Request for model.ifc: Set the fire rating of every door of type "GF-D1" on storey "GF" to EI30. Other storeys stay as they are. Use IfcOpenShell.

First a look at what the model holds.

```python
import ifcopenshell
import ifcopenshell.util.element

model = ifcopenshell.open("model.ifc")
print(model.schema)
storey = next(s for s in model.by_type("IfcBuildingStorey") if s.Name == "GF")
doors = [e for e in ifcopenshell.util.element.get_decomposition(storey) if e.is_a("IfcDoor")]
seen = {}
for e in doors:
    element_type = ifcopenshell.util.element.get_type(e)
    key = (element_type.Name if element_type != e and element_type else None, ifcopenshell.util.element.get_pset(e, "Pset_DoorCommon", "FireRating"))
    seen[key] = seen.get(key, 0) + 1
for (name, value), count in sorted(seen.items(), key=str):
    print(count, "x", name, "|", value)
```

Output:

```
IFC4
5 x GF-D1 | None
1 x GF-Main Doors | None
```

```python
import ifcopenshell
import ifcopenshell.api.pset
import ifcopenshell.util.element

model = ifcopenshell.open("model.ifc")

storey = next(s for s in model.by_type("IfcBuildingStorey") if s.Name == "GF")
doors = [e for e in ifcopenshell.util.element.get_decomposition(storey) if e.is_a("IfcDoor")]

count = 0
for e in doors:
    element_type = ifcopenshell.util.element.get_type(e)
    if element_type in (None, e) or element_type.Name != "GF-D1":
        continue
    # add_pset returns the element's existing set when there is one.
    pset = ifcopenshell.api.pset.add_pset(model, product=e, name="Pset_DoorCommon")
    ifcopenshell.api.pset.edit_pset(model, pset=pset, properties={"FireRating": "EI30"})
    count += 1

print(count, "doors updated")

model.write("model_rev.ifc")
```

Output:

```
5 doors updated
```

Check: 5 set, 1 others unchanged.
